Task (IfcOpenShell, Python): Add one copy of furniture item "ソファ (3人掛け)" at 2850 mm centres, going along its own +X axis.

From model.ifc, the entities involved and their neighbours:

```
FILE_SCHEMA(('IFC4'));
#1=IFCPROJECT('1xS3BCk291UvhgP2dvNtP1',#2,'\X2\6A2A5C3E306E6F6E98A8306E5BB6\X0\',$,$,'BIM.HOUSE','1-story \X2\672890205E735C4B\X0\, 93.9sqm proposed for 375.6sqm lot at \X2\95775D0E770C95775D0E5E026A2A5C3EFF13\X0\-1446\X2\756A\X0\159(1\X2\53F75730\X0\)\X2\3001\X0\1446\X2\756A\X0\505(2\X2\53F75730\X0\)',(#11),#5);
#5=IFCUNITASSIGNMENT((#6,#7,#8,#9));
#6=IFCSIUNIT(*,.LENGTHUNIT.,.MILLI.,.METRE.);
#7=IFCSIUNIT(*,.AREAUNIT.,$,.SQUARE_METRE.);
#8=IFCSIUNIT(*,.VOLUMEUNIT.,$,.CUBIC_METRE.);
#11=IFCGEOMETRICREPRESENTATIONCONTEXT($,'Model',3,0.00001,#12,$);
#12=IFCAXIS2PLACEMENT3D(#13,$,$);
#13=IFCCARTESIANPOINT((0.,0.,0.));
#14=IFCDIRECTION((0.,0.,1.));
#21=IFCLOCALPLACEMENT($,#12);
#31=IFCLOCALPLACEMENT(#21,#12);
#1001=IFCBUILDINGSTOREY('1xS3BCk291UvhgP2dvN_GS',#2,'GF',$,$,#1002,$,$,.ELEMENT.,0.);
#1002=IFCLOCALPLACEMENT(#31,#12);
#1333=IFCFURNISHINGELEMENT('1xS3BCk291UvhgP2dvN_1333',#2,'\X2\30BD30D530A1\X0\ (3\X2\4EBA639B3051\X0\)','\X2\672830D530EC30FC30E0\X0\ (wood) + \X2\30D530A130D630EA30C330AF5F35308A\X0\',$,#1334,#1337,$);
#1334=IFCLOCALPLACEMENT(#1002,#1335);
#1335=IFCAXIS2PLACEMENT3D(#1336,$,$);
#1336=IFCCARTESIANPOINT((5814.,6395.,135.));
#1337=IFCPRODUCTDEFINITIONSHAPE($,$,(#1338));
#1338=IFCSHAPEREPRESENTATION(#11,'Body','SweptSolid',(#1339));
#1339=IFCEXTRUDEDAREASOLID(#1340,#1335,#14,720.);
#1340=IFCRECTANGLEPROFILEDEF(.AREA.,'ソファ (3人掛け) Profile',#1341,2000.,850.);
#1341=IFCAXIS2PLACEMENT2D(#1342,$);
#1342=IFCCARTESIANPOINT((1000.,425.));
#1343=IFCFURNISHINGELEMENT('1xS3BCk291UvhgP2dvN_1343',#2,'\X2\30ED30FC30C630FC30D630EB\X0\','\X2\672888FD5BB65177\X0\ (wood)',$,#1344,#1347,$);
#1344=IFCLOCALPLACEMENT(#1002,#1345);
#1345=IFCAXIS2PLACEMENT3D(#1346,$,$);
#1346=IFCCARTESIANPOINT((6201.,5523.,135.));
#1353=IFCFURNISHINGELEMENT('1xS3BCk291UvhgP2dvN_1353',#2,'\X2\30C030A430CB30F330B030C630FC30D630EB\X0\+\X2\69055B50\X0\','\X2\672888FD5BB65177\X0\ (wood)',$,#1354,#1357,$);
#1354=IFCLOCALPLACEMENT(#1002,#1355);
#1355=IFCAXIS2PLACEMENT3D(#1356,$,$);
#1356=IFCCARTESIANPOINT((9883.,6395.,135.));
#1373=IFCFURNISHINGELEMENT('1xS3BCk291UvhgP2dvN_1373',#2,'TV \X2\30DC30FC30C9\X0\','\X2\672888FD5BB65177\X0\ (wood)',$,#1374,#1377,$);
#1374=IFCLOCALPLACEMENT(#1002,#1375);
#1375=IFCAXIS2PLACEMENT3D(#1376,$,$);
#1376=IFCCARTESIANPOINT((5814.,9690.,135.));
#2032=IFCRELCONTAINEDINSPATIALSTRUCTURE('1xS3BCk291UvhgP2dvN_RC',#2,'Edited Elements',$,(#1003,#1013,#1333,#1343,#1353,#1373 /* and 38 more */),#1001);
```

```python
import ifcopenshell
import ifcopenshell.api.geometry
import ifcopenshell.api.root
import ifcopenshell.util.element
import ifcopenshell.util.placement

model = ifcopenshell.open("model.ifc")


def reuse_history(source, copy):
    """copy_class also copies each property set's owner history, people and application; keep the originals."""
    for rel in copy.IsDefinedBy:
        if rel.is_a("IfcRelDefinesByProperties") and (history := rel.RelatingPropertyDefinition.OwnerHistory):
            rel.RelatingPropertyDefinition.OwnerHistory = source.OwnerHistory
            ifcopenshell.util.element.remove_deep2(model, history)


source = model.by_guid("1xS3BCk291UvhgP2dvN_1333")
base = ifcopenshell.util.placement.get_local_placement(source.ObjectPlacement)
step = base[:3, 0] * 2850.0

for i in range(1, 2):
    copy = ifcopenshell.api.root.copy_class(model, product=source)
    copy.Representation = ifcopenshell.util.element.copy_deep(
        model, source.Representation, exclude=["IfcGeometricRepresentationContext", "IfcRepresentationMap"]
    )
    reuse_history(source, copy)
    matrix = base.copy()
    matrix[:3, 3] += i * step
    print("added at", matrix[:3, 3].round(3) + 0.0)
    ifcopenshell.api.geometry.edit_object_placement(model, product=copy, matrix=matrix, is_si=False)

model.write("model_rev.ifc")
```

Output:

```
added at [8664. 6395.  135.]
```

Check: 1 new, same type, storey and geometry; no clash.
